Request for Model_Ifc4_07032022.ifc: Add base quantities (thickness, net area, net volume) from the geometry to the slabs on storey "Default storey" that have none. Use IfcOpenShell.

First a look at what the model holds.

```python
import ifcopenshell
import ifcopenshell.util.element
import ifcopenshell.util.unit

model = ifcopenshell.open("Model_Ifc4_07032022.ifc")
print(model.schema)
for unit_type in ("LENGTHUNIT", "AREAUNIT", "VOLUMEUNIT"):
    print(unit_type, ifcopenshell.util.unit.calculate_unit_scale(model, unit_type))
storey = next(s for s in model.by_type("IfcBuildingStorey") if s.Name == "Default storey")
slabs = [e for e in ifcopenshell.util.element.get_decomposition(storey) if e.is_a("IfcSlab")]
for e in sorted(slabs, key=lambda e: e.id()):
    print(e.id(), e.is_a(), e.Name, list(ifcopenshell.util.element.get_psets(e, qtos_only=True)), sep=" | ")
```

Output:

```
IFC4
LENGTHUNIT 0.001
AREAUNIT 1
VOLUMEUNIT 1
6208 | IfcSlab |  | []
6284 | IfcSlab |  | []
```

```python
import ifcopenshell
import ifcopenshell.api.pset
import ifcopenshell.geom
import ifcopenshell.util.element
import ifcopenshell.util.shape
import ifcopenshell.util.unit

model = ifcopenshell.open("Model_Ifc4_07032022.ifc")
unit_scale = ifcopenshell.util.unit.calculate_unit_scale(model)
area_scale = ifcopenshell.util.unit.calculate_unit_scale(model, "AREAUNIT")
volume_scale = ifcopenshell.util.unit.calculate_unit_scale(model, "VOLUMEUNIT")
settings = ifcopenshell.geom.settings()

storey = next(s for s in model.by_type("IfcBuildingStorey") if s.Name == "Default storey")
slabs = [e for e in ifcopenshell.util.element.get_decomposition(storey) if e.is_a("IfcSlab")]

for e in sorted(slabs, key=lambda e: e.id()):
    if ifcopenshell.util.element.get_psets(e, qtos_only=True, should_inherit=False):
        continue
    # Geometry comes back in metres, in the element's own axes.
    shape = ifcopenshell.geom.create_shape(settings, e)
    values = {
        "Width": ifcopenshell.util.shape.get_z(shape.geometry) / unit_scale,
        "NetArea": ifcopenshell.util.shape.get_footprint_area(shape.geometry) / area_scale,
        "NetVolume": ifcopenshell.util.shape.get_volume(shape.geometry) / volume_scale,
    }
    qto = ifcopenshell.api.pset.add_qto(model, product=e, name="Qto_SlabBaseQuantities")
    ifcopenshell.api.pset.edit_qto(model, qto=qto, properties=values)
    print(e.id(), {k: round(v, 3) for k, v in values.items()})

model.write("Model_Ifc4_07032022_rev.ifc")
```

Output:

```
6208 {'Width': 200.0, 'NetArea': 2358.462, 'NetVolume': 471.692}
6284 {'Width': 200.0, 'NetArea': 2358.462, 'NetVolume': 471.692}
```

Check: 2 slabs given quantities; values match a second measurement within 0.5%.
